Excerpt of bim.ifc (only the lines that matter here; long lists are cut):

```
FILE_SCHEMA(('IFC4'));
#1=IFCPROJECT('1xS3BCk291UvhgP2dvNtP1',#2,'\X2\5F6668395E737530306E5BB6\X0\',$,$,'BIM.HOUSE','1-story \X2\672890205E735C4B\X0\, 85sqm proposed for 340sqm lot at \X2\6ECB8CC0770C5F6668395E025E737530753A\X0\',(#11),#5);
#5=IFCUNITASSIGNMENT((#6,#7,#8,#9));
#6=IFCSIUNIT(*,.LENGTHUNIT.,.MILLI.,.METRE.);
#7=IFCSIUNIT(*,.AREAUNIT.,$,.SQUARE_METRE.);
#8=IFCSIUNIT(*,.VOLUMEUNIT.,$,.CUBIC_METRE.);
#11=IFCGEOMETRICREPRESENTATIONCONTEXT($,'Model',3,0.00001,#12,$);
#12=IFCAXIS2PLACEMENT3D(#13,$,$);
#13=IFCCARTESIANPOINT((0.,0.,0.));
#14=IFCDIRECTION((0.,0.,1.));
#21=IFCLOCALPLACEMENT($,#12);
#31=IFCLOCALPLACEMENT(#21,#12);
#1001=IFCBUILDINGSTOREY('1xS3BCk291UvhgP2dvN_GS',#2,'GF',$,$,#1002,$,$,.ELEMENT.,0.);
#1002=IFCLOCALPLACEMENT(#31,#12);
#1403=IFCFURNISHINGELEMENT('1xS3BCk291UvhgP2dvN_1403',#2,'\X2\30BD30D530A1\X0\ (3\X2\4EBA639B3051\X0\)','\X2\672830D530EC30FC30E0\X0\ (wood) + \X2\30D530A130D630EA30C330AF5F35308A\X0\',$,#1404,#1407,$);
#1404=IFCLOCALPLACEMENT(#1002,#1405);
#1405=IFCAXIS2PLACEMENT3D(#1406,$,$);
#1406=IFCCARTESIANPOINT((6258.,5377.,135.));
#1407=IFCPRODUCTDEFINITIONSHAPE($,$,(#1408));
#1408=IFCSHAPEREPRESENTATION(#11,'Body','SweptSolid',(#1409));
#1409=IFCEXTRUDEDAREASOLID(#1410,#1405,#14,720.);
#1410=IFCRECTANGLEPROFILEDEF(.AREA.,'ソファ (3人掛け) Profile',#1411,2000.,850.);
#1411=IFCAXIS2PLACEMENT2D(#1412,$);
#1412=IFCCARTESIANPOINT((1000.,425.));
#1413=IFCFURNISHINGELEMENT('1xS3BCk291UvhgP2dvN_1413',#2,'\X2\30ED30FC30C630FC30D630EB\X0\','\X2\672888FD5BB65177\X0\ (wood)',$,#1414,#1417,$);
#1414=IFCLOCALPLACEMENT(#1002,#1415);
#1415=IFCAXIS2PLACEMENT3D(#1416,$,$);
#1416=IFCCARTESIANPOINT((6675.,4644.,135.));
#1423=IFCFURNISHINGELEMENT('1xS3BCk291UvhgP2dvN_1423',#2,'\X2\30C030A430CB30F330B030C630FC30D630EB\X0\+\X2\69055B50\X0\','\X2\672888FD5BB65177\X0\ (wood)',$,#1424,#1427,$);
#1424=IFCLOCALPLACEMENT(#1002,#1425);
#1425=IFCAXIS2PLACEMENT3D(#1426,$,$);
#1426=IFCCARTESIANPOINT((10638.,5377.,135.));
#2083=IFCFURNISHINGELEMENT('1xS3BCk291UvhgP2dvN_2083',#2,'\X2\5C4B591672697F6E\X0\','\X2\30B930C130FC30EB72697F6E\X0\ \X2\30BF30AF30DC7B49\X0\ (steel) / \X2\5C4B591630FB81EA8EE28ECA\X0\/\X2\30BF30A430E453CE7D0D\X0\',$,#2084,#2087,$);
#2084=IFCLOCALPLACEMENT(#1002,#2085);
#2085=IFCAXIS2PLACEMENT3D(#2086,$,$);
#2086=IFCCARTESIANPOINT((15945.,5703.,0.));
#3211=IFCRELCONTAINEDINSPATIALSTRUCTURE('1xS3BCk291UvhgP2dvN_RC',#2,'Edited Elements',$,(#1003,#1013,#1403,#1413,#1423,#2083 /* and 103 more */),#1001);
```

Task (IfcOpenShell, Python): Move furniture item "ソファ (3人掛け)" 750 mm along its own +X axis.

```python
import ifcopenshell
import ifcopenshell.api.geometry
import ifcopenshell.util.placement
import ifcopenshell.util.unit

model = ifcopenshell.open("bim.ifc")
unit_scale = ifcopenshell.util.unit.calculate_unit_scale(model)

item = model.by_id(1403)
matrix = ifcopenshell.util.placement.get_local_placement(item.ObjectPlacement)
matrix[:3, 3] += matrix[:3, 0] * 0.75 / unit_scale
ifcopenshell.api.geometry.edit_object_placement(model, product=item, matrix=matrix, is_si=False)

print(ifcopenshell.util.placement.get_local_placement(item.ObjectPlacement).round(3) + 0.0)

model.write("bim_v2.ifc")
```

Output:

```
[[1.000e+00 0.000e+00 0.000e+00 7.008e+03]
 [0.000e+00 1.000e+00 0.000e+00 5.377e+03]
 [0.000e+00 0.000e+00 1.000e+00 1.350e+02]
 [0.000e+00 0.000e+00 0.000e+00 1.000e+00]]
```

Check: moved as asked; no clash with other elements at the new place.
